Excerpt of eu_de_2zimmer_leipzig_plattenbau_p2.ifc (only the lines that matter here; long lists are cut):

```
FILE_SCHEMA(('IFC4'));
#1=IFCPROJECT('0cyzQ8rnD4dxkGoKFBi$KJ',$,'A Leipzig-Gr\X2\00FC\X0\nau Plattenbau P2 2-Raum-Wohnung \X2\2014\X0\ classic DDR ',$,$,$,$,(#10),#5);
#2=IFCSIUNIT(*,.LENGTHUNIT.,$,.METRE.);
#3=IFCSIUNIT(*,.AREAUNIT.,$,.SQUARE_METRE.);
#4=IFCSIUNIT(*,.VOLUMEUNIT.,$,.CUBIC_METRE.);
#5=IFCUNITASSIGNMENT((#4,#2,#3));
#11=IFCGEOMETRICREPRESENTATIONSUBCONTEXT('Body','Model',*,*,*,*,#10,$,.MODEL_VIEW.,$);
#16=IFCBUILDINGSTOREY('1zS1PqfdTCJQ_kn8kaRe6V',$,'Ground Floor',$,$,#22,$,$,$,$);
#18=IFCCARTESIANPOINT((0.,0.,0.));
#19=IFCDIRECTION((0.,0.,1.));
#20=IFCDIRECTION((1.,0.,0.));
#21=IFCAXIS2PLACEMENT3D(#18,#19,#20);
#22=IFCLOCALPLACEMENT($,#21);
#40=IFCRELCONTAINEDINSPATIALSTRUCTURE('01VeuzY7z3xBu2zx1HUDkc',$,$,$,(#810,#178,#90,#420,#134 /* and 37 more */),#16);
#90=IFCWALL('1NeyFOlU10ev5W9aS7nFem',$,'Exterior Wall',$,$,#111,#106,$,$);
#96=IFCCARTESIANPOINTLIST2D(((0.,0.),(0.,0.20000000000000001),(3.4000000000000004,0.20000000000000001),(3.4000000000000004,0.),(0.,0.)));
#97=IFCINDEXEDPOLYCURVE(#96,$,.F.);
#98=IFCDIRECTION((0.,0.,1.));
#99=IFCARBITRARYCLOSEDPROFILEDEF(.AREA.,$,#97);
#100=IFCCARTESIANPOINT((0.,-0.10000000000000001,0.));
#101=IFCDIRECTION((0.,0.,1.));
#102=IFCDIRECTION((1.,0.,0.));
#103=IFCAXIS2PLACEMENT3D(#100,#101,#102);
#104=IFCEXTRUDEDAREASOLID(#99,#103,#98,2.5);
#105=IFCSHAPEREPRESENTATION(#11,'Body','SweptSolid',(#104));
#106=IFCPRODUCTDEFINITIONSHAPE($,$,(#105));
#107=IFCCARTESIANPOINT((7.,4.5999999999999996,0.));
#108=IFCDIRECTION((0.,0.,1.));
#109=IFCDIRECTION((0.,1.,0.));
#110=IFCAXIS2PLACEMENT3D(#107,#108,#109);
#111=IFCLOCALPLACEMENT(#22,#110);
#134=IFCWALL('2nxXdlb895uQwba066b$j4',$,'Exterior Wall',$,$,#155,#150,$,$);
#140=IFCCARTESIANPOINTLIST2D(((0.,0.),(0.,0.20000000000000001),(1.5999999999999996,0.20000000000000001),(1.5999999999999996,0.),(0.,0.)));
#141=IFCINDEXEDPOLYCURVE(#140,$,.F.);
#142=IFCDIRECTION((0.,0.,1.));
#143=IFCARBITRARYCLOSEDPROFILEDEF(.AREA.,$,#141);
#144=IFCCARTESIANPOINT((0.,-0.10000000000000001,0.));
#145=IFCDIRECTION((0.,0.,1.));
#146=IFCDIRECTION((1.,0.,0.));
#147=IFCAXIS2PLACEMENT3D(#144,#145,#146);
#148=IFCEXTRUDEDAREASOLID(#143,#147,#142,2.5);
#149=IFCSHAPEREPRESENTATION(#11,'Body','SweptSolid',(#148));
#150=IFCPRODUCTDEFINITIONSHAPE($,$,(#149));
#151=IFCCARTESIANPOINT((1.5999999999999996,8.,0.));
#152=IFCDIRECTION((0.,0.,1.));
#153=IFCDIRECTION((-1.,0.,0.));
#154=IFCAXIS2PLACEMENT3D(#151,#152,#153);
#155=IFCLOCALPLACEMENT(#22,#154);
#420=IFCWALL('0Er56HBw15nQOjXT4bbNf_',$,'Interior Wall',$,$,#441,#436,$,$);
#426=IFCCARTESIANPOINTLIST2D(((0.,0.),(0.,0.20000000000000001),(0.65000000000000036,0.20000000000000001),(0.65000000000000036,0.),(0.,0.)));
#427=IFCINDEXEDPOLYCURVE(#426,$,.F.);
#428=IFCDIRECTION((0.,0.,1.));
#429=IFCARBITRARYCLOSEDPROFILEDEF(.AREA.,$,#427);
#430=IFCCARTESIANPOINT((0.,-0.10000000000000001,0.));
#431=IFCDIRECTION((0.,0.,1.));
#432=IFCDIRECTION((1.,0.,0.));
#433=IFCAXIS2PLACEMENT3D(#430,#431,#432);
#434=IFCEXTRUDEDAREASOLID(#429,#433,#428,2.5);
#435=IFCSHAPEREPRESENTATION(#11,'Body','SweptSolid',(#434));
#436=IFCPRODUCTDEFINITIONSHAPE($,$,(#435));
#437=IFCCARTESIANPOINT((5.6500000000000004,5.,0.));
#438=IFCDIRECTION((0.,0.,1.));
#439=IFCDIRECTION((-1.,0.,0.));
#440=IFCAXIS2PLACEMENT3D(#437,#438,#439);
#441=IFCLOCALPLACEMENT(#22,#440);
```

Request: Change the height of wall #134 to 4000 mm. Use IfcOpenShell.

```python
import ifcopenshell
import ifcopenshell.geom
import ifcopenshell.util.representation
import ifcopenshell.util.shape
import ifcopenshell.util.unit

model = ifcopenshell.open("eu_de_2zimmer_leipzig_plattenbau_p2.ifc")
unit_scale = ifcopenshell.util.unit.calculate_unit_scale(model)
settings = ifcopenshell.geom.settings()


def volume(element):
    """Net volume in cubic metres, openings subtracted."""
    shape = ifcopenshell.geom.create_shape(settings, element)
    return ifcopenshell.util.shape.get_volume(shape.geometry)


wall = model.by_guid("2nxXdlb895uQwba066b$j4")
before = volume(wall)

body = ifcopenshell.util.representation.get_representation(wall, "Model", "Body")
solid = body.Items[0]
old_height = solid.Depth
solid.Depth = 4 / unit_scale
after = volume(wall)

print(f"height {old_height:g} -> {solid.Depth:g}, volume {before:.3f} -> {after:.3f} m3")

model.write("eu_de_2zimmer_leipzig_plattenbau_p2_rev.ifc")
```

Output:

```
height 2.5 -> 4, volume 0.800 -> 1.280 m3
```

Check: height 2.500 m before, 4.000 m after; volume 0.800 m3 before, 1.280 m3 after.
